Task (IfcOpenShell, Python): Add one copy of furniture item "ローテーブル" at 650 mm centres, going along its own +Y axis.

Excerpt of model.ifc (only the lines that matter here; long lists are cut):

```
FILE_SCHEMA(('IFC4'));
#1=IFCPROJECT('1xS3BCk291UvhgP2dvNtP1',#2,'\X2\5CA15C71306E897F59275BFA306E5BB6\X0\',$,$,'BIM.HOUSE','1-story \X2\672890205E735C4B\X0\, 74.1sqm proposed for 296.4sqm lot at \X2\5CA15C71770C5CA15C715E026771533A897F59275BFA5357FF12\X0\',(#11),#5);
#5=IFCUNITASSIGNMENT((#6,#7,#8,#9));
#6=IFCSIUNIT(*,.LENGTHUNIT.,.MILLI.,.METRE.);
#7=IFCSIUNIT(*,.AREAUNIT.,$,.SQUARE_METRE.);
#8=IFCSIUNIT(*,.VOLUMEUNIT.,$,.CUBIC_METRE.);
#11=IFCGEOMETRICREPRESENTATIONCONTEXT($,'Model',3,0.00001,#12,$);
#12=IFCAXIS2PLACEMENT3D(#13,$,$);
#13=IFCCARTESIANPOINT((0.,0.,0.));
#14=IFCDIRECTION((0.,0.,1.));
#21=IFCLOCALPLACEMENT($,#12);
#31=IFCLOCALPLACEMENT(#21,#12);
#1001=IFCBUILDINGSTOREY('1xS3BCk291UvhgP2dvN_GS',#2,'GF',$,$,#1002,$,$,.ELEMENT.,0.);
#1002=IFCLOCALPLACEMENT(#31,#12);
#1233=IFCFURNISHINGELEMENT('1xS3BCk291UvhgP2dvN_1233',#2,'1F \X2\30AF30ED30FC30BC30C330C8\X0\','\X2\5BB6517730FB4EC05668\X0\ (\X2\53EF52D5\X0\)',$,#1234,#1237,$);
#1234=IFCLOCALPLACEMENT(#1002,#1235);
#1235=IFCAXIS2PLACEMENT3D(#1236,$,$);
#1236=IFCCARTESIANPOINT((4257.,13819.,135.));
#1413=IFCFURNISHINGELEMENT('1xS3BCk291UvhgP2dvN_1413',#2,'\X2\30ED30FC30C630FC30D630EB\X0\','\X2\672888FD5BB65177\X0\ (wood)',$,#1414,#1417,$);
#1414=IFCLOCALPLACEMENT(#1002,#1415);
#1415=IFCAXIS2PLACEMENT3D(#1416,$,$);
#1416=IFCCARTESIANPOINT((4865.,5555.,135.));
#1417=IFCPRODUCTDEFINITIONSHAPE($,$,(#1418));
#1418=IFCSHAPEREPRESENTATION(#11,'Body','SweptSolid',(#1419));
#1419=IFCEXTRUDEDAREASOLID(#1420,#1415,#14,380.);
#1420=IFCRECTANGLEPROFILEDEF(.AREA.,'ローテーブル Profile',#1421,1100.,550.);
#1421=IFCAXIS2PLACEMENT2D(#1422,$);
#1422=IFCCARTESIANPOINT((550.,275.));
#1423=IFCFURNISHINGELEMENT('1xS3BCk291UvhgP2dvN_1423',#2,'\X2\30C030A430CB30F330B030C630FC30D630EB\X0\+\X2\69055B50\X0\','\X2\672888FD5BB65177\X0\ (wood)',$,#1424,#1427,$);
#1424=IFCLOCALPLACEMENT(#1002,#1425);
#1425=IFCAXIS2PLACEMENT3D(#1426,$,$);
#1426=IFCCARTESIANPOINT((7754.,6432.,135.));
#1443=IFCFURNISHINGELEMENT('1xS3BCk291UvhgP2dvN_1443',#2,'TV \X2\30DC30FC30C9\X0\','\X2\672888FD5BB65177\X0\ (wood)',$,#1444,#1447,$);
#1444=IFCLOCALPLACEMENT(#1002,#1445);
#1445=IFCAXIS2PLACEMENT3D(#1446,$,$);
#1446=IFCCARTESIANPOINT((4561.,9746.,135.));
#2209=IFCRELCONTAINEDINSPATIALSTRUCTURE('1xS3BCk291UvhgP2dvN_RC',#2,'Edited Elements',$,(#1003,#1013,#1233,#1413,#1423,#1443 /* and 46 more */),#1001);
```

```python
import ifcopenshell
import ifcopenshell.api.geometry
import ifcopenshell.api.root
import ifcopenshell.util.element
import ifcopenshell.util.placement
import ifcopenshell.util.unit

model = ifcopenshell.open("model.ifc")
unit_scale = ifcopenshell.util.unit.calculate_unit_scale(model)


def reuse_history(source, copy):
    """copy_class also copies each property set's owner history, people and application; keep the originals."""
    for rel in copy.IsDefinedBy:
        if rel.is_a("IfcRelDefinesByProperties") and (history := rel.RelatingPropertyDefinition.OwnerHistory):
            rel.RelatingPropertyDefinition.OwnerHistory = source.OwnerHistory
            ifcopenshell.util.element.remove_deep2(model, history)


source = model.by_id(1413)
base = ifcopenshell.util.placement.get_local_placement(source.ObjectPlacement)
step = base[:3, 1] * 0.65 / unit_scale

for i in range(1, 2):
    copy = ifcopenshell.api.root.copy_class(model, product=source)
    copy.Representation = ifcopenshell.util.element.copy_deep(
        model, source.Representation, exclude=["IfcGeometricRepresentationContext", "IfcRepresentationMap"]
    )
    reuse_history(source, copy)
    matrix = base.copy()
    matrix[:3, 3] += i * step
    print("added at", matrix[:3, 3].round(3) + 0.0)
    ifcopenshell.api.geometry.edit_object_placement(model, product=copy, matrix=matrix, is_si=False)

model.write("model-out.ifc")
```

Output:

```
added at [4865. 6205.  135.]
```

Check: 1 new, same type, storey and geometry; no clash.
